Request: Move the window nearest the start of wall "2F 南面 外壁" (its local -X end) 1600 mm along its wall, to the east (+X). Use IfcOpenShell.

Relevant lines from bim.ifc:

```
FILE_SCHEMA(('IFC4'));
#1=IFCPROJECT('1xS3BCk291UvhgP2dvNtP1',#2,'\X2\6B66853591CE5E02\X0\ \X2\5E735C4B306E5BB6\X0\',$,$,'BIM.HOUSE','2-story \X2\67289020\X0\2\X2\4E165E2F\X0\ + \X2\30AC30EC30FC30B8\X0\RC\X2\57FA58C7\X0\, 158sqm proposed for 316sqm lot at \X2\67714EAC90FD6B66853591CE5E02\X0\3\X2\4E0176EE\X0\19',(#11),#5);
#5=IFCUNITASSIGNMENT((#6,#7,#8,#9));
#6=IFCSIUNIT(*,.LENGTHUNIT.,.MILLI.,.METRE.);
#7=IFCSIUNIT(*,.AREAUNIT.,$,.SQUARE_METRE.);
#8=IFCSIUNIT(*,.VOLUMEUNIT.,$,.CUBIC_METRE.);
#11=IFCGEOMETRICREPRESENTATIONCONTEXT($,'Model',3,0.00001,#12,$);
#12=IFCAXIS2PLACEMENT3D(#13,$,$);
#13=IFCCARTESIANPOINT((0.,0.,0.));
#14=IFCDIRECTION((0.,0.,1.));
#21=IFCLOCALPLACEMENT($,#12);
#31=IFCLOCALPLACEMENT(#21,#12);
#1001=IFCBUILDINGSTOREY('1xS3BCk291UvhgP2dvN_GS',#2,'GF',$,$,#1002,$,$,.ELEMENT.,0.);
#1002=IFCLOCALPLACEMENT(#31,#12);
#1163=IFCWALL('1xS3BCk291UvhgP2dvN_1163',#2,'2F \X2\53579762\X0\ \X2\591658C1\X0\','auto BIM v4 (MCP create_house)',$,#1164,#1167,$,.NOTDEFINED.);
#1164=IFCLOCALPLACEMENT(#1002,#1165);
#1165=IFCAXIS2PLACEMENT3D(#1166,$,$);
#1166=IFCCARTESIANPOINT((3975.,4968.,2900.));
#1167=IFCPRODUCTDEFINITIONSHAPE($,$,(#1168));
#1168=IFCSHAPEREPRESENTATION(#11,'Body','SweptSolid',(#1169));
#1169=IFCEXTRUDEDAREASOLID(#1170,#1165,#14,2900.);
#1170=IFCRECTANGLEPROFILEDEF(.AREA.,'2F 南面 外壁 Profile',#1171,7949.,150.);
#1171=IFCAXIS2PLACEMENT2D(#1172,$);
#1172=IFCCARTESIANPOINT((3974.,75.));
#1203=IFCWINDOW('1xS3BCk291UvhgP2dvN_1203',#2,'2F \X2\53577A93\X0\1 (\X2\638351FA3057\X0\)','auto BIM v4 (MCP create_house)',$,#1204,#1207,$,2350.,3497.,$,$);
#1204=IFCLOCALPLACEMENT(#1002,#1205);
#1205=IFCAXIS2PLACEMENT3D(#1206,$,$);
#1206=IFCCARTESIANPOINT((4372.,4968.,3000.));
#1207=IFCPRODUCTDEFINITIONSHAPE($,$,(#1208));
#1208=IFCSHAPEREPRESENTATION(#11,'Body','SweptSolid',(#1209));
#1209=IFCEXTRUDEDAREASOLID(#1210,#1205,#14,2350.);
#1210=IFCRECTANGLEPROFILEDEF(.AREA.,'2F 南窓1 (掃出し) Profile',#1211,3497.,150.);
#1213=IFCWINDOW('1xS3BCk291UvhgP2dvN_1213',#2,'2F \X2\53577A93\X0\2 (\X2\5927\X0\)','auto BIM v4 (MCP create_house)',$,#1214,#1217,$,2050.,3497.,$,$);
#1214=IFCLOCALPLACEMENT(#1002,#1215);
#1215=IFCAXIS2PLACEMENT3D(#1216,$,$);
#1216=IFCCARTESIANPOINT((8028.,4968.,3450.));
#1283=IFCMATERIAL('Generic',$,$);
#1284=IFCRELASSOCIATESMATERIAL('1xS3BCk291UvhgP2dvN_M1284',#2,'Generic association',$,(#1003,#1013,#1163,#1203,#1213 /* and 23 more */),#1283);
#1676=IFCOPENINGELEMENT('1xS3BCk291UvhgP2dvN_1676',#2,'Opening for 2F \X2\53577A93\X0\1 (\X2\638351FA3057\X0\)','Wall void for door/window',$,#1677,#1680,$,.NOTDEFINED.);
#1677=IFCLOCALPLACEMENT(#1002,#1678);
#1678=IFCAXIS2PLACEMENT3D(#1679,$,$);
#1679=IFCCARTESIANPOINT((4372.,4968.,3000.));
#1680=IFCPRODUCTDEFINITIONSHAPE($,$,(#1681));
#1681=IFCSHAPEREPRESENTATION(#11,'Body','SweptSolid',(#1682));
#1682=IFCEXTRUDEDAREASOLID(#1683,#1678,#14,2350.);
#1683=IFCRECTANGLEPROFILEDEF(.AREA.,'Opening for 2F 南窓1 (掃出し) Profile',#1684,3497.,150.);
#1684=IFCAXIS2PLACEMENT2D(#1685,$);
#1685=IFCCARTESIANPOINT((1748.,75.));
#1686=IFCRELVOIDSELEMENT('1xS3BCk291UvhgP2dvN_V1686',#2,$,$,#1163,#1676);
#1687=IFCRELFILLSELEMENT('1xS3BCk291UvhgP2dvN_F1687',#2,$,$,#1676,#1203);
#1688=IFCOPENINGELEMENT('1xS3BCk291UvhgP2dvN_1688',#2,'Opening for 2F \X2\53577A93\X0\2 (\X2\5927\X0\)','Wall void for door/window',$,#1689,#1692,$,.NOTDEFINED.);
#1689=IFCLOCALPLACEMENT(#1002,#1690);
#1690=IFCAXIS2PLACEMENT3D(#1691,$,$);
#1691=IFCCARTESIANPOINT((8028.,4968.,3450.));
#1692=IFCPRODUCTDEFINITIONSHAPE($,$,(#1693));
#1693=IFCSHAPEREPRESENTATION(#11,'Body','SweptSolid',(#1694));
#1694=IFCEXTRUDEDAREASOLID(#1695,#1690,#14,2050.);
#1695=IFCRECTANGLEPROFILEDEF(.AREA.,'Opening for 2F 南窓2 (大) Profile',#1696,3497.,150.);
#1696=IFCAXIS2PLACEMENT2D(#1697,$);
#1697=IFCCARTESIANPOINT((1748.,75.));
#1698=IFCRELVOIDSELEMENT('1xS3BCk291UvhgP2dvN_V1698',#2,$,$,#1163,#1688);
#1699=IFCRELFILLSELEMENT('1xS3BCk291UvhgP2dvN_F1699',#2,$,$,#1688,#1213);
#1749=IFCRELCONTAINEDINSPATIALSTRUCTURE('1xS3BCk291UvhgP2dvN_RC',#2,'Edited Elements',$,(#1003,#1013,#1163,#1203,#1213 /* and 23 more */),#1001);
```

```python
import ifcopenshell
import ifcopenshell.api.geometry
import ifcopenshell.util.placement
import ifcopenshell.util.unit

model = ifcopenshell.open("bim.ifc")
unit_scale = ifcopenshell.util.unit.calculate_unit_scale(model)

window = model.by_id(1203)
opening = window.FillsVoids[0].RelatingOpeningElement
wall = opening.VoidsElements[0].RelatingBuildingElement

wall_matrix = ifcopenshell.util.placement.get_local_placement(wall.ObjectPlacement)
shift = wall_matrix[:3, 0] * 1.6 / unit_scale
before = ifcopenshell.util.placement.get_local_placement(window.ObjectPlacement)[:3, 3].copy()

# The window is not placed relative to its opening, so move both.
for product in (opening, window):
    matrix = ifcopenshell.util.placement.get_local_placement(product.ObjectPlacement)
    matrix[:3, 3] += shift
    ifcopenshell.api.geometry.edit_object_placement(model, product=product, matrix=matrix, is_si=False)

after = ifcopenshell.util.placement.get_local_placement(window.ObjectPlacement)[:3, 3]
print("window moved by", (after - before).round(3) + 0.0)

model.write("bim_edited.ifc")
```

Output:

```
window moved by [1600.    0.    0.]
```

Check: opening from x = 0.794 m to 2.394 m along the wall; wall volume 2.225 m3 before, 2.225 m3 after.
